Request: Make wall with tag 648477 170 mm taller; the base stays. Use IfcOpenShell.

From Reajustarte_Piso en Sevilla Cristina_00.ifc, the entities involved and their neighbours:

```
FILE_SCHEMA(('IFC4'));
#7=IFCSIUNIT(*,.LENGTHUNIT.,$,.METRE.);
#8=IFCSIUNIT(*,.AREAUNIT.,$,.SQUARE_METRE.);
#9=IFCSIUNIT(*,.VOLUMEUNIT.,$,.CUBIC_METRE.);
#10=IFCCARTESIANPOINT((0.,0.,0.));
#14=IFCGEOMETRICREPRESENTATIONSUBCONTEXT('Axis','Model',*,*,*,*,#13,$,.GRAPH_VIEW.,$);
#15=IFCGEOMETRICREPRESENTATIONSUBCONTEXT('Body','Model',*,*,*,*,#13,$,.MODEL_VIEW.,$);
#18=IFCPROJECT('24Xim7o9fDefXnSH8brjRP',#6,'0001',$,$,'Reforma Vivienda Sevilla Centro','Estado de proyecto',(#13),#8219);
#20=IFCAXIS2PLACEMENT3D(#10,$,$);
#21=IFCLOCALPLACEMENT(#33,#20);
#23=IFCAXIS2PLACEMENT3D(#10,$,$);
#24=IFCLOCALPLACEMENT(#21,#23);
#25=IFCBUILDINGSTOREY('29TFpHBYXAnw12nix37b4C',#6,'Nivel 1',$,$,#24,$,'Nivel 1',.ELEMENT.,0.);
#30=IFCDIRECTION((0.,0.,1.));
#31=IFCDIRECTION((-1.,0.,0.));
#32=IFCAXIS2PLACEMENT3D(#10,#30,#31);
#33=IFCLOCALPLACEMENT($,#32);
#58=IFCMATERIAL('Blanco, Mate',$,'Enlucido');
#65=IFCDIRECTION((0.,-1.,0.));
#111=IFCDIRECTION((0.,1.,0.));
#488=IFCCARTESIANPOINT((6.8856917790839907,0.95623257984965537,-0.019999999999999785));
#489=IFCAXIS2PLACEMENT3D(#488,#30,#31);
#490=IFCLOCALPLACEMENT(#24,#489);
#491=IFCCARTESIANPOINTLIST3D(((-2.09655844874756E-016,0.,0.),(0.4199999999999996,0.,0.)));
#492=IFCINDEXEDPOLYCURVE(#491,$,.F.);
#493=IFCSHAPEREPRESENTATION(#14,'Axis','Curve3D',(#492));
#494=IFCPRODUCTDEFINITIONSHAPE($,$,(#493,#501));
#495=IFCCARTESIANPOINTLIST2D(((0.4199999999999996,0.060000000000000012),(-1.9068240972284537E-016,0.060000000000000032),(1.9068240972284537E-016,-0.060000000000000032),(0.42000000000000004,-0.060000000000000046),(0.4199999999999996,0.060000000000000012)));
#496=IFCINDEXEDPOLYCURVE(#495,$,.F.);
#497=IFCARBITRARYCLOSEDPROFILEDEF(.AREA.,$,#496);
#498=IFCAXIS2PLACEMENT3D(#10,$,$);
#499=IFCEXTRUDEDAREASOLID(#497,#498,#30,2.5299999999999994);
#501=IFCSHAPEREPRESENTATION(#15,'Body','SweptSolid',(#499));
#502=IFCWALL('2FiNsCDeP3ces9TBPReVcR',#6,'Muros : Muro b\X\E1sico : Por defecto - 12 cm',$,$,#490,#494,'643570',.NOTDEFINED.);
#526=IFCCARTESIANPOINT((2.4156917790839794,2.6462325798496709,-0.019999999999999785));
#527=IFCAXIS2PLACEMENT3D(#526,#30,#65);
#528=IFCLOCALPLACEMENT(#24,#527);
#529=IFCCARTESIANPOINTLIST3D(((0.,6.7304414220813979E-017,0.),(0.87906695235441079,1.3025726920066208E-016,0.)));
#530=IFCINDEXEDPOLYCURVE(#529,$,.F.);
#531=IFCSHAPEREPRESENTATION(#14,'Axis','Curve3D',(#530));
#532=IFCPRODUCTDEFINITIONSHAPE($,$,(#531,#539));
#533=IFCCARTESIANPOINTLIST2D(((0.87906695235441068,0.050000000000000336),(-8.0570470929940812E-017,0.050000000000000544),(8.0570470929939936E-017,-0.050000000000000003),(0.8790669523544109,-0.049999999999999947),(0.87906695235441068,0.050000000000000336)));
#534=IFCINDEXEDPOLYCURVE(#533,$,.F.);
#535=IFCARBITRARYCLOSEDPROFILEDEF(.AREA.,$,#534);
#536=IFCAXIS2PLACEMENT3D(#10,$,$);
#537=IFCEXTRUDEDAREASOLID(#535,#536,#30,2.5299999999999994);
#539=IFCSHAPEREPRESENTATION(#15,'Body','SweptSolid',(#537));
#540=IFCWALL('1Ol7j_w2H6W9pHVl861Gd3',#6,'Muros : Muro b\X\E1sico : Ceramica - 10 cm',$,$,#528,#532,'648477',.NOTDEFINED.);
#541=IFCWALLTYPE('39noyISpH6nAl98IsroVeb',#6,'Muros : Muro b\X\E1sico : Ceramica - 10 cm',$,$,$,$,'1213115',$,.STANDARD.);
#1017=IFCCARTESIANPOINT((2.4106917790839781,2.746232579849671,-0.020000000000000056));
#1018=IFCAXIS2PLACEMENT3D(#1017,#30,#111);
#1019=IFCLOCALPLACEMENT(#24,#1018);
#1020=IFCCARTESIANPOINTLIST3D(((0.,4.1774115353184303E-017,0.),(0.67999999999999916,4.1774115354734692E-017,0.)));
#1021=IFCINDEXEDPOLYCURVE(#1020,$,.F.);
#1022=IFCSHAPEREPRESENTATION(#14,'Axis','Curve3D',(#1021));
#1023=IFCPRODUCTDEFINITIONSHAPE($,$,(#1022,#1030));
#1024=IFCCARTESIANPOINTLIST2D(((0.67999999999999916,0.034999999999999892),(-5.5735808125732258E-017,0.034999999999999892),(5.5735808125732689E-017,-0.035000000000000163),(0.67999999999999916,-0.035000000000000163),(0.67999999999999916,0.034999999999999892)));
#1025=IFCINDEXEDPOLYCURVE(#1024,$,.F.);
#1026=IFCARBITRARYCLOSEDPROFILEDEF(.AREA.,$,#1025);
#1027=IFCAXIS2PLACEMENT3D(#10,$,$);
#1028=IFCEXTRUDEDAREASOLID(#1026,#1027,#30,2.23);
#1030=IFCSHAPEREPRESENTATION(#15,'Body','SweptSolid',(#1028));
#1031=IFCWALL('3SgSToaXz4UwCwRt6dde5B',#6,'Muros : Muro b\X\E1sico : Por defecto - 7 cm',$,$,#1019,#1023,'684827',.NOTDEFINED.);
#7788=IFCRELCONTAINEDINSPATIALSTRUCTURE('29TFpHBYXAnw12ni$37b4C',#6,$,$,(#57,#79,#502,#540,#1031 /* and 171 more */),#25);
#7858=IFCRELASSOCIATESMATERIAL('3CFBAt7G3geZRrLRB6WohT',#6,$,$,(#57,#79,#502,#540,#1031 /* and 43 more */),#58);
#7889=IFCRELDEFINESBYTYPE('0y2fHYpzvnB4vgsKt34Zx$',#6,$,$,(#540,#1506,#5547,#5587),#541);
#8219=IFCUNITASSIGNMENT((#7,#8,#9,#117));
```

```python
import ifcopenshell
import ifcopenshell.geom
import ifcopenshell.util.representation
import ifcopenshell.util.shape
import ifcopenshell.util.unit

model = ifcopenshell.open("Reajustarte_Piso en Sevilla Cristina_00.ifc")
unit_scale = ifcopenshell.util.unit.calculate_unit_scale(model)
settings = ifcopenshell.geom.settings()


def volume(element):
    """Net volume in cubic metres, openings subtracted."""
    shape = ifcopenshell.geom.create_shape(settings, element)
    return ifcopenshell.util.shape.get_volume(shape.geometry)


wall = model.by_guid("1Ol7j_w2H6W9pHVl861Gd3")
before = volume(wall)

body = ifcopenshell.util.representation.get_representation(wall, "Model", "Body")
solid = body.Items[0]
old_height = solid.Depth
solid.Depth += 0.17 / unit_scale
after = volume(wall)

print(f"height {old_height:g} -> {solid.Depth:g}, volume {before:.3f} -> {after:.3f} m3")

model.write("Reajustarte_Piso en Sevilla Cristina_00_updated.ifc")
```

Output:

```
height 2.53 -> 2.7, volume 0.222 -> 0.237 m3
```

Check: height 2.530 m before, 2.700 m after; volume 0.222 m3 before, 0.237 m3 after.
